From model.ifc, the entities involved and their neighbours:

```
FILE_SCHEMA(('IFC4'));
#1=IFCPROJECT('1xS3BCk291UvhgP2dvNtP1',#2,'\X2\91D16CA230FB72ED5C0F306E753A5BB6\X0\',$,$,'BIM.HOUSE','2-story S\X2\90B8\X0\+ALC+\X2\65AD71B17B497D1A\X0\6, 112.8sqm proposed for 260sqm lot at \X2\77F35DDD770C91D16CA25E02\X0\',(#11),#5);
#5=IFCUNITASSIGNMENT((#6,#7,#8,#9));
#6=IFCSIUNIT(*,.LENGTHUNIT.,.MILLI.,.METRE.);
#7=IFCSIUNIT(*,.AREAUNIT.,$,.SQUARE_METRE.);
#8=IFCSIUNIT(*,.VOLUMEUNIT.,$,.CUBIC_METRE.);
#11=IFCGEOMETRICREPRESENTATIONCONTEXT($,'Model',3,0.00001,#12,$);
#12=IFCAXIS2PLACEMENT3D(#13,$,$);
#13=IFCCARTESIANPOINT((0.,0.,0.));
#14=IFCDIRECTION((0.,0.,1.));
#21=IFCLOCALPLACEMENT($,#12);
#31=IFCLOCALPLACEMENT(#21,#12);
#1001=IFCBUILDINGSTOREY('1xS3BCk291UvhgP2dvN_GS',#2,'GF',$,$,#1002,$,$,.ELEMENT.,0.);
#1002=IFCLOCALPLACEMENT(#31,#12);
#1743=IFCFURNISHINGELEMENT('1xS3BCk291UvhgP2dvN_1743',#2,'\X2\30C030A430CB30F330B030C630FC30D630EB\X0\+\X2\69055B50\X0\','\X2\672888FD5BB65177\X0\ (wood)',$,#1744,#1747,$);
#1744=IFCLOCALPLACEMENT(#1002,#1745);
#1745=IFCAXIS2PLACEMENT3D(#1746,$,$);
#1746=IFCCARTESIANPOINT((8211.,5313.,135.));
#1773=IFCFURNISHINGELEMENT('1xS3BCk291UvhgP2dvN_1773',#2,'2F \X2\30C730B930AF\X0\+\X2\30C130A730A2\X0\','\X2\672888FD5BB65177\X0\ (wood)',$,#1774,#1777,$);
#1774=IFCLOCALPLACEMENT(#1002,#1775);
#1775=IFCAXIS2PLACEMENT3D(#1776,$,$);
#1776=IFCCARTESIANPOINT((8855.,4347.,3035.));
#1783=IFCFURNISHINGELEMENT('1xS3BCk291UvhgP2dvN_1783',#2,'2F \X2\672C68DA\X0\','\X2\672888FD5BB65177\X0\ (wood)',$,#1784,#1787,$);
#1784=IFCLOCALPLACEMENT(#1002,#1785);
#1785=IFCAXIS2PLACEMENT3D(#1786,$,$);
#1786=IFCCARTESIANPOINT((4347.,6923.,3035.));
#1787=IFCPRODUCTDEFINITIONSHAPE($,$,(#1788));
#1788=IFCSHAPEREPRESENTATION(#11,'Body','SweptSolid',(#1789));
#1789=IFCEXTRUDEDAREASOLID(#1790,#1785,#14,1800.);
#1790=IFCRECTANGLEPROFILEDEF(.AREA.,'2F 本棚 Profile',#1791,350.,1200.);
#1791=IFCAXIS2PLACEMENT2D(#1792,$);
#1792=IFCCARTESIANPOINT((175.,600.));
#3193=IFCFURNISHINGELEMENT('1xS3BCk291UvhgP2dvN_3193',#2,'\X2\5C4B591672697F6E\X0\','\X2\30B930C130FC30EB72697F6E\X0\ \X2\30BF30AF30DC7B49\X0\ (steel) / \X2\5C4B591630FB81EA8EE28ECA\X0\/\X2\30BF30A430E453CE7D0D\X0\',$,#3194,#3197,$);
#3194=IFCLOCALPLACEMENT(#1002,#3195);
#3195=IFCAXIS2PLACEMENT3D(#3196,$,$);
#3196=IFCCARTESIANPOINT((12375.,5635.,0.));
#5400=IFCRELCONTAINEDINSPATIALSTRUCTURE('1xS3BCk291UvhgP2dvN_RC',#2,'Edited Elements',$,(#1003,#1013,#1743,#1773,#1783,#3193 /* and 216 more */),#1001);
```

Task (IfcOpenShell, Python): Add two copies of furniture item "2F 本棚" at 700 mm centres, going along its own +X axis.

```python
import ifcopenshell
import ifcopenshell.api.geometry
import ifcopenshell.api.root
import ifcopenshell.util.element
import ifcopenshell.util.placement

model = ifcopenshell.open("model.ifc")


def reuse_history(source, copy):
    """copy_class also copies each property set's owner history, people and application; keep the originals."""
    for rel in copy.IsDefinedBy:
        if rel.is_a("IfcRelDefinesByProperties") and (history := rel.RelatingPropertyDefinition.OwnerHistory):
            rel.RelatingPropertyDefinition.OwnerHistory = source.OwnerHistory
            ifcopenshell.util.element.remove_deep2(model, history)


source = model.by_guid("1xS3BCk291UvhgP2dvN_1783")
base = ifcopenshell.util.placement.get_local_placement(source.ObjectPlacement)
step = base[:3, 0] * 700.0

for i in range(1, 3):
    copy = ifcopenshell.api.root.copy_class(model, product=source)
    copy.Representation = ifcopenshell.util.element.copy_deep(
        model, source.Representation, exclude=["IfcGeometricRepresentationContext", "IfcRepresentationMap"]
    )
    reuse_history(source, copy)
    matrix = base.copy()
    matrix[:3, 3] += i * step
    print("added at", matrix[:3, 3].round(3) + 0.0)
    ifcopenshell.api.geometry.edit_object_placement(model, product=copy, matrix=matrix, is_si=False)

model.write("model_rev.ifc")
```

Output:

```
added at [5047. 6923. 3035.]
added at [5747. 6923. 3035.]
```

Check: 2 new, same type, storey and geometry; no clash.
